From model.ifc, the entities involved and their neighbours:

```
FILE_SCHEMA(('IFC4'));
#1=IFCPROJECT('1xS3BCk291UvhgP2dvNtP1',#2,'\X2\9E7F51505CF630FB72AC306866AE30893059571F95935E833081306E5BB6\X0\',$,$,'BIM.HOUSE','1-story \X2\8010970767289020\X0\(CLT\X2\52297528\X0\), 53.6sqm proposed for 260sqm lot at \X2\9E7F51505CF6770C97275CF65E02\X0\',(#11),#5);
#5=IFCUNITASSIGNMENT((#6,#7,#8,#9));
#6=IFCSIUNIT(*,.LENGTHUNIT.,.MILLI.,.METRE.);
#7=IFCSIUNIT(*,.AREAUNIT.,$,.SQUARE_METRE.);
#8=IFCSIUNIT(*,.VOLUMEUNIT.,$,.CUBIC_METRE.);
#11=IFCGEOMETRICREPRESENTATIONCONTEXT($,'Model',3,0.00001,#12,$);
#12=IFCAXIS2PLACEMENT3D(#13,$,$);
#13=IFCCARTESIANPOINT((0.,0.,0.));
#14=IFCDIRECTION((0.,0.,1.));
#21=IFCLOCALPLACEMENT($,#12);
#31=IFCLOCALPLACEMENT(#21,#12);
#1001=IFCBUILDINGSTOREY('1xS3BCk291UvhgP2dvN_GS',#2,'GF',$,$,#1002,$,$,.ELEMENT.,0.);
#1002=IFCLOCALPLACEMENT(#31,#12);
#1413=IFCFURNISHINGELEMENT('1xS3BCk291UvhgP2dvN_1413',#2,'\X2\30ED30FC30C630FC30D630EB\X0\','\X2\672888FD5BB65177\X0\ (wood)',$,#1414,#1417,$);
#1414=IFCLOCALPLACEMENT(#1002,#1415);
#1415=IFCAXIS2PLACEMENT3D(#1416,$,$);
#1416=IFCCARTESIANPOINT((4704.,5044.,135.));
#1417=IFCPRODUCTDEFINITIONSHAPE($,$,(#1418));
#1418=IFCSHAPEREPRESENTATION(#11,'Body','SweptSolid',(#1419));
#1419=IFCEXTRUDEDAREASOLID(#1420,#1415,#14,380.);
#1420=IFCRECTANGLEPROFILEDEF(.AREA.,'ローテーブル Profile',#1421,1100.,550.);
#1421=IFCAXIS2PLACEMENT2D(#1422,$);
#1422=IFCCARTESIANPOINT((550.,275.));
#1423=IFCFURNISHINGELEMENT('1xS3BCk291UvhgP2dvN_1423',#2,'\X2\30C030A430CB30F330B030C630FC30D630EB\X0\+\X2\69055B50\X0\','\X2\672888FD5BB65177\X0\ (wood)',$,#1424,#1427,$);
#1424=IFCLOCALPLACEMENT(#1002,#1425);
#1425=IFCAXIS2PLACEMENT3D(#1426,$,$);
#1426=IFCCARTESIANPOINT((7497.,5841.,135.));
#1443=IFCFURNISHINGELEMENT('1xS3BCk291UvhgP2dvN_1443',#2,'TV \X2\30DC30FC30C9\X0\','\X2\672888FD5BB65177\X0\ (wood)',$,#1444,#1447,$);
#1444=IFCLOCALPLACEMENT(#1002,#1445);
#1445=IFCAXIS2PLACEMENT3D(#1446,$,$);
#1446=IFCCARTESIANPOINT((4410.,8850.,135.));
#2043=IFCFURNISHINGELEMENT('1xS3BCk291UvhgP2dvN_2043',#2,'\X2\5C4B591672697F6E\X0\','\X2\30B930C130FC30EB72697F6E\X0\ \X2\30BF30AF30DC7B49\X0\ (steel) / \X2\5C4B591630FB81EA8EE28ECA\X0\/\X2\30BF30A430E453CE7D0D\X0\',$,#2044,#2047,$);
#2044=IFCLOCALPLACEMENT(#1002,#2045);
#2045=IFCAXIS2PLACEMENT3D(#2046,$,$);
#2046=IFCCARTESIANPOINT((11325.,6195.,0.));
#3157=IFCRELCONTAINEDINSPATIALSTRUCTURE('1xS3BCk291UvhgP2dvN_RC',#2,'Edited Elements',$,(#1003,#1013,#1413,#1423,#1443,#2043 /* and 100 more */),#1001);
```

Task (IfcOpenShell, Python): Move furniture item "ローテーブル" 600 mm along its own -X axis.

```python
import ifcopenshell
import ifcopenshell.api.geometry
import ifcopenshell.util.placement
import ifcopenshell.util.unit

model = ifcopenshell.open("model.ifc")
unit_scale = ifcopenshell.util.unit.calculate_unit_scale(model)

item = model.by_id(1413)
matrix = ifcopenshell.util.placement.get_local_placement(item.ObjectPlacement)
matrix[:3, 3] -= matrix[:3, 0] * 0.6 / unit_scale
ifcopenshell.api.geometry.edit_object_placement(model, product=item, matrix=matrix, is_si=False)

print(ifcopenshell.util.placement.get_local_placement(item.ObjectPlacement).round(3) + 0.0)

model.write("model-out.ifc")
```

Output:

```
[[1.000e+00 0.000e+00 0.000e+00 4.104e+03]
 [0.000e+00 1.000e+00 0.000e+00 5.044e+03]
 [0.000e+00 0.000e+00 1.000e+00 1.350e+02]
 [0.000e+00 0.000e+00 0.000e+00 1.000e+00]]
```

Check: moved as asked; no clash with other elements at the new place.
